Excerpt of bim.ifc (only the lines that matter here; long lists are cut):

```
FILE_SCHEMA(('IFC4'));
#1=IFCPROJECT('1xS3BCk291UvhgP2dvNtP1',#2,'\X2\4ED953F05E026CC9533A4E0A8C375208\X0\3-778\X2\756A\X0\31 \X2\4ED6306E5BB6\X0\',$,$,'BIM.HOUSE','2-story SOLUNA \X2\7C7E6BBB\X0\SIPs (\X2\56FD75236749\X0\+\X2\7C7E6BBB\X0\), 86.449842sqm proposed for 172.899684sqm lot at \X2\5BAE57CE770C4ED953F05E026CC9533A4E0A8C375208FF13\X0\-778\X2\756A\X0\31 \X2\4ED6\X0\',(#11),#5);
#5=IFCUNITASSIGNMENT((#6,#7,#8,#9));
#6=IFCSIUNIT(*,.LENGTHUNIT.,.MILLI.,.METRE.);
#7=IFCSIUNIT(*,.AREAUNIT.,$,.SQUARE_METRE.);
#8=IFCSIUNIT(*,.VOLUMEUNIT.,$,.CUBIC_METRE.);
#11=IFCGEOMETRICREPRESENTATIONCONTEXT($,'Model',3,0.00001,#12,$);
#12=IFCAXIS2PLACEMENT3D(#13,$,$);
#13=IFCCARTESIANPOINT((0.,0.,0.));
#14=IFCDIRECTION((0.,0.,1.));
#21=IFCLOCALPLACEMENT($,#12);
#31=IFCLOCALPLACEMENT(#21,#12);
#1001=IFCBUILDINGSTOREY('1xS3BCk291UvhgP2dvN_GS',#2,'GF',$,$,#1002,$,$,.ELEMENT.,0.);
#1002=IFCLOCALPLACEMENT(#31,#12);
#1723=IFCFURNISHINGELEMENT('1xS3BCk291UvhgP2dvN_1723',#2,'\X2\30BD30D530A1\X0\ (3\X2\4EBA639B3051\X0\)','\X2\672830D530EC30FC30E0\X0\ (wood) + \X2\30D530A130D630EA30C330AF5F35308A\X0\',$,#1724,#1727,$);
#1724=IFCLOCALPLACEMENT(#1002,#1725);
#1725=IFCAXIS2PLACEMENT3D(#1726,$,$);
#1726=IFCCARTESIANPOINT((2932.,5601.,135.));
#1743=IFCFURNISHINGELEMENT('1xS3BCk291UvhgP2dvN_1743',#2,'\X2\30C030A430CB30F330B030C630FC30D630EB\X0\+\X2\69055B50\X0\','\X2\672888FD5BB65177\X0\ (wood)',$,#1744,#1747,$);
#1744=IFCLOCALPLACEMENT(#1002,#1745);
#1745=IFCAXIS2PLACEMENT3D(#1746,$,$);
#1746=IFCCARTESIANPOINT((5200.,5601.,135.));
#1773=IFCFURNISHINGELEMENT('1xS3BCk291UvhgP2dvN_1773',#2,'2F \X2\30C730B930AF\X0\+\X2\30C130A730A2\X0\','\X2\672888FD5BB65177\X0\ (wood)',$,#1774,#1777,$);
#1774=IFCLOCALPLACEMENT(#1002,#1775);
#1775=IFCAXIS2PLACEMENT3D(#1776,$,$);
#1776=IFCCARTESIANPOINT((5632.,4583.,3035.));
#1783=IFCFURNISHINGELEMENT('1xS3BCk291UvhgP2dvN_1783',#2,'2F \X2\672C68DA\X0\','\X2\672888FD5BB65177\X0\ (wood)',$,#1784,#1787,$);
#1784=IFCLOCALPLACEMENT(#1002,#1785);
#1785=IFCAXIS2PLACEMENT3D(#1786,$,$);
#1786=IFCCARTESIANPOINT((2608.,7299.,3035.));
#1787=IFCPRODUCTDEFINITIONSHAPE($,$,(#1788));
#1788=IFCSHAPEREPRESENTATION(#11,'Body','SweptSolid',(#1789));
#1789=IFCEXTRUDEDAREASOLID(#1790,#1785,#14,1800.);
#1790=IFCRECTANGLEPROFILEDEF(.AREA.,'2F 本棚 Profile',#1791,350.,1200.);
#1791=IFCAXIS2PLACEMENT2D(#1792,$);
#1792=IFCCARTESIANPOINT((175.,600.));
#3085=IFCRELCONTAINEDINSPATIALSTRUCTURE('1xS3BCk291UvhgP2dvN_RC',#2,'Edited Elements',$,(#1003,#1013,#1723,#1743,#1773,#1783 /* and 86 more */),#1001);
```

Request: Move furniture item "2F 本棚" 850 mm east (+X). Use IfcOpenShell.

```python
import ifcopenshell
import ifcopenshell.api.geometry
import ifcopenshell.util.placement
import ifcopenshell.util.unit

model = ifcopenshell.open("bim.ifc")
unit_scale = ifcopenshell.util.unit.calculate_unit_scale(model)

item = model.by_guid("1xS3BCk291UvhgP2dvN_1783")
matrix = ifcopenshell.util.placement.get_local_placement(item.ObjectPlacement)
matrix[0, 3] += 0.85 / unit_scale
ifcopenshell.api.geometry.edit_object_placement(model, product=item, matrix=matrix, is_si=False)

print(ifcopenshell.util.placement.get_local_placement(item.ObjectPlacement).round(3) + 0.0)

model.write("bim_updated.ifc")
```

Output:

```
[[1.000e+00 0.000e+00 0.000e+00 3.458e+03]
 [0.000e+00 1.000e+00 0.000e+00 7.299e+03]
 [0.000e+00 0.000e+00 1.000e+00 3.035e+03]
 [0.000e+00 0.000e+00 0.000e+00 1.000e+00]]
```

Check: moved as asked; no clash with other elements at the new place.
